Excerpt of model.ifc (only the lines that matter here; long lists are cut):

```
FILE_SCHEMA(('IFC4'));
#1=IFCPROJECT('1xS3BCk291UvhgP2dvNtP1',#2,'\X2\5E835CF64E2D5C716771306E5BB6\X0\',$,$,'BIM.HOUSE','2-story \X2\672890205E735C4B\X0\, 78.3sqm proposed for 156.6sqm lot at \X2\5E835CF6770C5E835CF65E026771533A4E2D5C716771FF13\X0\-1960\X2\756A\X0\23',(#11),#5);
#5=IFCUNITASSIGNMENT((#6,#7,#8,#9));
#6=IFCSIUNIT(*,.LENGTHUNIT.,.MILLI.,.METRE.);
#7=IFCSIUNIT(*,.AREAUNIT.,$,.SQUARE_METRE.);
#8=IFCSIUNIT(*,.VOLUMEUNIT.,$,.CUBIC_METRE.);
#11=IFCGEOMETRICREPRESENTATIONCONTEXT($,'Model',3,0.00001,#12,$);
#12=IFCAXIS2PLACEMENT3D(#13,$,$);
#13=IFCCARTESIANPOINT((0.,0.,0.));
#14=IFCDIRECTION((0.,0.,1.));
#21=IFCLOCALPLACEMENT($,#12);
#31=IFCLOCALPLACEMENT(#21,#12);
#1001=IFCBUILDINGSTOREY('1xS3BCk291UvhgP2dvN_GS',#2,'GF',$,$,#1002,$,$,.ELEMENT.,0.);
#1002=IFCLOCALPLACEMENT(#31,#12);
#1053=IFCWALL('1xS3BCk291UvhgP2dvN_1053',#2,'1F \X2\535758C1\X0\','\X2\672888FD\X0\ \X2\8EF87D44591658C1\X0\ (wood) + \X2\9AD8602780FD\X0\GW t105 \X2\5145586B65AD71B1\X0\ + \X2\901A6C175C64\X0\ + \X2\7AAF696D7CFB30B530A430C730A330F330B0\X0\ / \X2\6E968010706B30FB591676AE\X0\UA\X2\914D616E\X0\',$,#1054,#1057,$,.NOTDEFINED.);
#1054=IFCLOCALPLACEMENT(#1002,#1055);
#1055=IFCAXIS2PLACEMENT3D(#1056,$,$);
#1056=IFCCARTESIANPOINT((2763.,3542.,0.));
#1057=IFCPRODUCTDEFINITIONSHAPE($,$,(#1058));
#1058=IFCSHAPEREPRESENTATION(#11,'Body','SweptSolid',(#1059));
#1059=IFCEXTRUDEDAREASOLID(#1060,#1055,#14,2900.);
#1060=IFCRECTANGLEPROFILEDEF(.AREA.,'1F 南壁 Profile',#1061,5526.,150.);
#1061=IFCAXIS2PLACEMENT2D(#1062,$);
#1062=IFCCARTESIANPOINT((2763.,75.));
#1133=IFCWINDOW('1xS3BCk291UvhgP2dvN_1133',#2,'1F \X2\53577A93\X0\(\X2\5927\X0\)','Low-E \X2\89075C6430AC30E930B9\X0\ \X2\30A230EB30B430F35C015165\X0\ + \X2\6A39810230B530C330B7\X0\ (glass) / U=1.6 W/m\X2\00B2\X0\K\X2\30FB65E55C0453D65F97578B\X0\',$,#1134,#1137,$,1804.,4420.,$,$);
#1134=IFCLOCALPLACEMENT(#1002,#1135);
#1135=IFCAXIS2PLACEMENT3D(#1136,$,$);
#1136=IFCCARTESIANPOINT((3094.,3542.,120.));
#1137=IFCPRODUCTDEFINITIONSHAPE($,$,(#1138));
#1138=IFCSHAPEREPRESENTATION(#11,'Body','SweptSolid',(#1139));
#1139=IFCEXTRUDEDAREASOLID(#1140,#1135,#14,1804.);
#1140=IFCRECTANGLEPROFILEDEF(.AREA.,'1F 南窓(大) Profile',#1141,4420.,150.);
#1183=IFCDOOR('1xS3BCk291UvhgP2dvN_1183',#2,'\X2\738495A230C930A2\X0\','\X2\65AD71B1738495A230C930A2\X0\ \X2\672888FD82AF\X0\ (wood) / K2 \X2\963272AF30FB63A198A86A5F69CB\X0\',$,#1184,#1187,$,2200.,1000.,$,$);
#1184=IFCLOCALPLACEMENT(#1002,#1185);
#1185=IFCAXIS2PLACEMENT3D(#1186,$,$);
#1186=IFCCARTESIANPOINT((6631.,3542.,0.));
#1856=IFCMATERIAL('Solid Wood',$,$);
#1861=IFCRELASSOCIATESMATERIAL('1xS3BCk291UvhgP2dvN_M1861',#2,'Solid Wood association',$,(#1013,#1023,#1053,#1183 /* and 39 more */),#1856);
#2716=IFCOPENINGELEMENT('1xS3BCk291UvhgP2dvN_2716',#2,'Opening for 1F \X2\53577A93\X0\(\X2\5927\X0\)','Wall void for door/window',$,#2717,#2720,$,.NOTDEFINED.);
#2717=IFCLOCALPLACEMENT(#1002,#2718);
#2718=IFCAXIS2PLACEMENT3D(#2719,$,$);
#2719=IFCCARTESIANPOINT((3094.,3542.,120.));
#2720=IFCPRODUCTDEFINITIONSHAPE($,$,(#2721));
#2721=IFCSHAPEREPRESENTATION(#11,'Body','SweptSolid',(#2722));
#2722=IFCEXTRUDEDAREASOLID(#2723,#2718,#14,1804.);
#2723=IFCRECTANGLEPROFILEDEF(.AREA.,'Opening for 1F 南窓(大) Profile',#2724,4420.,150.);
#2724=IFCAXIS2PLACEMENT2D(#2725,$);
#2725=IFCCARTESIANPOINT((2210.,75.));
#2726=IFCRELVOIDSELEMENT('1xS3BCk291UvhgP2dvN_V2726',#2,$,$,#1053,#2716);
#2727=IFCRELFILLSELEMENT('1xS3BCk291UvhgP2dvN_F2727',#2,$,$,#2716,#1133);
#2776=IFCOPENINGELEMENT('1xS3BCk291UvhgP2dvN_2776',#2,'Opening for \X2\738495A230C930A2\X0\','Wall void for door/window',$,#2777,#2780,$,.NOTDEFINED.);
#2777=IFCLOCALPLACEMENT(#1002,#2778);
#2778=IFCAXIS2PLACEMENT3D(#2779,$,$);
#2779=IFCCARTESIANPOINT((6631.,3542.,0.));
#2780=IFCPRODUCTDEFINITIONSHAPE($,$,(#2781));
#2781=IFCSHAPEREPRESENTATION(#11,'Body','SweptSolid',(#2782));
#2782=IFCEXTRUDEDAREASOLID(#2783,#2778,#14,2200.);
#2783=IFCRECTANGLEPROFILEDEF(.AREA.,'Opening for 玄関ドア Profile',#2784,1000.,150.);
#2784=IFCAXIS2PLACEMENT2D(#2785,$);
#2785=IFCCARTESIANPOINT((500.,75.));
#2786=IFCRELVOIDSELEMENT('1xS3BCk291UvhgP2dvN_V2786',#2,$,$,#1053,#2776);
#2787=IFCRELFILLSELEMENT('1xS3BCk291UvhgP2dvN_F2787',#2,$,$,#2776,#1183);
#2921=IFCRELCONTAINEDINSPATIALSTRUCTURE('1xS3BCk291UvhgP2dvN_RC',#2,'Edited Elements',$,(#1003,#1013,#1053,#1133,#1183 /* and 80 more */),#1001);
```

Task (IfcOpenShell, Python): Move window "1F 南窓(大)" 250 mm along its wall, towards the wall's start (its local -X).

```python
import ifcopenshell
import ifcopenshell.api.geometry
import ifcopenshell.util.placement
import ifcopenshell.util.unit

model = ifcopenshell.open("model.ifc")
unit_scale = ifcopenshell.util.unit.calculate_unit_scale(model)

window = model.by_id(1133)
opening = window.FillsVoids[0].RelatingOpeningElement
wall = opening.VoidsElements[0].RelatingBuildingElement

wall_matrix = ifcopenshell.util.placement.get_local_placement(wall.ObjectPlacement)
shift = wall_matrix[:3, 0] * -0.25 / unit_scale
before = ifcopenshell.util.placement.get_local_placement(window.ObjectPlacement)[:3, 3].copy()

# The window is not placed relative to its opening, so move both.
for product in (opening, window):
    matrix = ifcopenshell.util.placement.get_local_placement(product.ObjectPlacement)
    matrix[:3, 3] += shift
    ifcopenshell.api.geometry.edit_object_placement(model, product=product, matrix=matrix, is_si=False)

after = ifcopenshell.util.placement.get_local_placement(window.ObjectPlacement)[:3, 3]
print("window moved by", (after - before).round(3) + 0.0)

model.write("model_v2.ifc")
```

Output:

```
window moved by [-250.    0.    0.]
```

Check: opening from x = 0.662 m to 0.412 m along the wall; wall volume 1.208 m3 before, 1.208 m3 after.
